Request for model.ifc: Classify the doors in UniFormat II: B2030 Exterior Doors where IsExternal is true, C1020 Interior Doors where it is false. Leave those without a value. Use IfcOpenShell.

First a look at what the model holds.

```python
import ifcopenshell
import ifcopenshell.util.element

model = ifcopenshell.open("model.ifc")
print(model.schema)
print("classifications:", [c.Name for c in model.by_type("IfcClassification")])
values = [ifcopenshell.util.element.get_pset(e, "Pset_DoorCommon", "IsExternal") for e in model.by_type("IfcDoor")]
for value in (True, False, None):
    print("IsExternal", value, values.count(value))
```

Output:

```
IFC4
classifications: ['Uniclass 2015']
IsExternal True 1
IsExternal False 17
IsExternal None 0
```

```python
import ifcopenshell
import ifcopenshell.api.classification
import ifcopenshell.util.element

model = ifcopenshell.open("model.ifc")

system = ifcopenshell.api.classification.add_classification(model, classification="UniFormat II")

doors = model.by_type("IfcDoor")
external = {e: ifcopenshell.util.element.get_pset(e, "Pset_DoorCommon", "IsExternal") for e in doors}
for flag, code, name in ((True, "B2030", "Exterior Doors"), (False, "C1020", "Interior Doors")):
    products = [e for e in doors if external[e] is flag]
    ifcopenshell.api.classification.add_reference(
        model, products=products, classification=system, identification=code, name=name
    )
    print(code, len(products))

model.write("model_edited.ifc")
```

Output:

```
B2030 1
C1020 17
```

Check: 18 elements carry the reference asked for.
